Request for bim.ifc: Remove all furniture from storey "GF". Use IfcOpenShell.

First a look at what the model holds.

```python
import ifcopenshell
import ifcopenshell.util.element

model = ifcopenshell.open("bim.ifc")
print(model.schema)
storey = next(s for s in model.by_type("IfcBuildingStorey") if s.Name == "GF")
furniture = [e for e in ifcopenshell.util.element.get_decomposition(storey) if e.is_a("IfcFurnishingElement")]
seen = {}
for e in furniture:
    element_type = ifcopenshell.util.element.get_type(e)
    name = element_type.Name if element_type not in (None, e) else None
    seen[name] = seen.get(name, 0) + 1
for name, count in sorted(seen.items(), key=str):
    print(count, "x", name)
```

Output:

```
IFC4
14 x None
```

```python
import ifcopenshell
import ifcopenshell.api.root
import ifcopenshell.util.element

model = ifcopenshell.open("bim.ifc")

storey = next(s for s in model.by_type("IfcBuildingStorey") if s.Name == "GF")
furniture = [e for e in ifcopenshell.util.element.get_decomposition(storey) if e.is_a("IfcFurnishingElement")]

for e in furniture:
    ifcopenshell.api.root.remove_product(model, product=e)
print(len(furniture), "removed")

model.write("bim_v2.ifc")
```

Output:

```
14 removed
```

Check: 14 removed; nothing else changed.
